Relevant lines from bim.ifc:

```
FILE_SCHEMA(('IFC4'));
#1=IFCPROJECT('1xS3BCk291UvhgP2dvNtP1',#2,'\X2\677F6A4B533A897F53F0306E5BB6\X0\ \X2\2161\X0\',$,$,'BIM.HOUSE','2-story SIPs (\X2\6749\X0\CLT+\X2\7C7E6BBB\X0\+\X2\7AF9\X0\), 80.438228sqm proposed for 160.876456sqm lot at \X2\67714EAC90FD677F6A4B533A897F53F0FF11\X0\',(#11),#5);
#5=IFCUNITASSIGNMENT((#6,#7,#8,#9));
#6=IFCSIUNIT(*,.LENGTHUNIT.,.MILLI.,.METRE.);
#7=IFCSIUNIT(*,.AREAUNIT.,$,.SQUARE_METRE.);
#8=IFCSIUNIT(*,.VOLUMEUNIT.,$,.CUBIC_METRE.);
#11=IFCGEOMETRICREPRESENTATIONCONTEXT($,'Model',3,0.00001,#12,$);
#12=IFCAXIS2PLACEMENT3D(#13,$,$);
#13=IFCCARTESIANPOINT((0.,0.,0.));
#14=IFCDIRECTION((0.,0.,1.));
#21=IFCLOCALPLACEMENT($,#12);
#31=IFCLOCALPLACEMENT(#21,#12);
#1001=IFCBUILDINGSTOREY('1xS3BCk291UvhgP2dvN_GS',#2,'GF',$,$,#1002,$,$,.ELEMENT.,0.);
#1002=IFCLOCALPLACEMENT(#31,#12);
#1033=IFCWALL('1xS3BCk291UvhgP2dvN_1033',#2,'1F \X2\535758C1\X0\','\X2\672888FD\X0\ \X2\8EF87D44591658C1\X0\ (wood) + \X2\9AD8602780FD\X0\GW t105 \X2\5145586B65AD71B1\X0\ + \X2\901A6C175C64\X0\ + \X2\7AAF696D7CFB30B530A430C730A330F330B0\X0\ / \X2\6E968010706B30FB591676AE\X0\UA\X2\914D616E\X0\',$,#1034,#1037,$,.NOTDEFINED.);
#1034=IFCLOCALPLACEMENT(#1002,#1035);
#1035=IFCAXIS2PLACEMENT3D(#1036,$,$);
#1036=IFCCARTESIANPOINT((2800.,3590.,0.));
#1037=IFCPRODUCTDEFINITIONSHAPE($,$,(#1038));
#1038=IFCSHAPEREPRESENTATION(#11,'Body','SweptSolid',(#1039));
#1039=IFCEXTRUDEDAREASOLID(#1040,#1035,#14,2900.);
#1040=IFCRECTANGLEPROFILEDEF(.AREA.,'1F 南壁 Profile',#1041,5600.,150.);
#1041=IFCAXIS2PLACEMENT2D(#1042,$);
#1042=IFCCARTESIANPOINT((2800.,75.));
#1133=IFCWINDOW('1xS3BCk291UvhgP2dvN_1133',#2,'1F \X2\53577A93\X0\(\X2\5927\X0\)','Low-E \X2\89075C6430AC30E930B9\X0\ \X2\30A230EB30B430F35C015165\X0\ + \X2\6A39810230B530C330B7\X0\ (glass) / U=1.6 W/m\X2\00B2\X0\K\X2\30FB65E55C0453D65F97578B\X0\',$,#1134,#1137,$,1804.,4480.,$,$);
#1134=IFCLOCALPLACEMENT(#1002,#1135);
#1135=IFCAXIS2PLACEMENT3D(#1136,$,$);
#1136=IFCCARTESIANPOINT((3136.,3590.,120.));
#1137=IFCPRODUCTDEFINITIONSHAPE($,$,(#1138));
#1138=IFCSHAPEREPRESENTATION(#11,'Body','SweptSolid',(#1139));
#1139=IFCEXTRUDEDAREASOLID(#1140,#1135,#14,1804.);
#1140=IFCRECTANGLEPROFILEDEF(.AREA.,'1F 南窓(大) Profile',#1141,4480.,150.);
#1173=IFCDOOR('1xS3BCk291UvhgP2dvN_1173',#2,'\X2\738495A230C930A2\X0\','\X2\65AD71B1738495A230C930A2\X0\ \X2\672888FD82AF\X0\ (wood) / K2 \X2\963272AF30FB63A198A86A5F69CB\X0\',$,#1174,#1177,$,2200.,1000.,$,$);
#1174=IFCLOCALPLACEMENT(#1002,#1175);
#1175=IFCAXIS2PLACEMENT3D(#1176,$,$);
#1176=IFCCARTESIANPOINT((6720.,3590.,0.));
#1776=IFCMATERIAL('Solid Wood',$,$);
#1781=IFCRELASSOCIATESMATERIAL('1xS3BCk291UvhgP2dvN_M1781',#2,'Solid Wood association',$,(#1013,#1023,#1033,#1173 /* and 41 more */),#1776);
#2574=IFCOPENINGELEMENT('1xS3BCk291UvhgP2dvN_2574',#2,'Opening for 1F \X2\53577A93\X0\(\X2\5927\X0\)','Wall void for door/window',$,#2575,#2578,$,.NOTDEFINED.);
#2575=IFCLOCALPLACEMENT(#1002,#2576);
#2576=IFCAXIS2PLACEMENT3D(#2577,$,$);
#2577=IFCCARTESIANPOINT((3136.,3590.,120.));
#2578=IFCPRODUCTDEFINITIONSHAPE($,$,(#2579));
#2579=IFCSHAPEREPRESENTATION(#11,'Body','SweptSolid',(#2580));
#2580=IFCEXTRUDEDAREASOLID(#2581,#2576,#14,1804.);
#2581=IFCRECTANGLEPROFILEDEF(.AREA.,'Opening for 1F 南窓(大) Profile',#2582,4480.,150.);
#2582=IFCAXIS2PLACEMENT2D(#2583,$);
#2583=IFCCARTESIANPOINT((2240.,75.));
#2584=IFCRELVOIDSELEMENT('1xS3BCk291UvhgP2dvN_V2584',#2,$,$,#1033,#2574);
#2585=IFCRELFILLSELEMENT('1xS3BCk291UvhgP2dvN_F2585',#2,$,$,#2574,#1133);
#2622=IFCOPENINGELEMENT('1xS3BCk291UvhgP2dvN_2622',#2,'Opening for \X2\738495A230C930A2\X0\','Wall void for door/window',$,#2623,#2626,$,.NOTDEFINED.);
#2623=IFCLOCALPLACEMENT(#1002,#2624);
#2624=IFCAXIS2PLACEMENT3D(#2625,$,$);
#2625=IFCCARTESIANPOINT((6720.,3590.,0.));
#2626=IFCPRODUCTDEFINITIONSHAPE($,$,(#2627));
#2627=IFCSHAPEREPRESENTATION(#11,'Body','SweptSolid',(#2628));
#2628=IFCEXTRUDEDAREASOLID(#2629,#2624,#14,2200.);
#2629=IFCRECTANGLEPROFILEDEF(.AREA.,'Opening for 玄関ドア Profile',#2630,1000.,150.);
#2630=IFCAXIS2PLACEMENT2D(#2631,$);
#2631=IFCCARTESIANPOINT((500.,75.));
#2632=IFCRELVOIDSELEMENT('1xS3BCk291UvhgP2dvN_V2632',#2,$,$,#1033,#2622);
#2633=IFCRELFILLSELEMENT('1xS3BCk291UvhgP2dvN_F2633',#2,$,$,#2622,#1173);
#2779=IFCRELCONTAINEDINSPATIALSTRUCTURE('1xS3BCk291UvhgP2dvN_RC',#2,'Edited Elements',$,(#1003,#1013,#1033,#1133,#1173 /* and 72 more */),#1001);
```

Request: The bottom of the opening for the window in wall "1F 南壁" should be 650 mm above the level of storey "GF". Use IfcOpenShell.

```python
import numpy as np
import ifcopenshell
import ifcopenshell.api.geometry
import ifcopenshell.geom
import ifcopenshell.util.element
import ifcopenshell.util.placement
import ifcopenshell.util.shape
import ifcopenshell.util.unit

model = ifcopenshell.open("bim.ifc")
unit_scale = ifcopenshell.util.unit.calculate_unit_scale(model)

window = model.by_id(1133)
opening = window.FillsVoids[0].RelatingOpeningElement
storey = ifcopenshell.util.element.get_container(window, ifc_class="IfcBuildingStorey")
level = ifcopenshell.util.placement.get_local_placement(storey.ObjectPlacement)[2, 3]

# The opening's origin need not be at the sill, so measure its lowest point.
shape = ifcopenshell.geom.create_shape(ifcopenshell.geom.settings(), opening)
bottom = ifcopenshell.util.shape.get_shape_bottom_elevation(shape, shape.geometry) / unit_scale
dz = level + 650.0 - bottom

shift = np.array([0.0, 0.0, dz])
# The window is not placed relative to its opening, so move both.
for product in (opening, window):
    matrix = ifcopenshell.util.placement.get_local_placement(product.ObjectPlacement)
    matrix[:3, 3] += shift
    ifcopenshell.api.geometry.edit_object_placement(model, product=product, matrix=matrix, is_si=False)

print(f"moved by {dz * unit_scale:+.3f} m")

model.write("bim_v2.ifc")
```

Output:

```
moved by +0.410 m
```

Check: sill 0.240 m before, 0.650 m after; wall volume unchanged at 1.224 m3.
